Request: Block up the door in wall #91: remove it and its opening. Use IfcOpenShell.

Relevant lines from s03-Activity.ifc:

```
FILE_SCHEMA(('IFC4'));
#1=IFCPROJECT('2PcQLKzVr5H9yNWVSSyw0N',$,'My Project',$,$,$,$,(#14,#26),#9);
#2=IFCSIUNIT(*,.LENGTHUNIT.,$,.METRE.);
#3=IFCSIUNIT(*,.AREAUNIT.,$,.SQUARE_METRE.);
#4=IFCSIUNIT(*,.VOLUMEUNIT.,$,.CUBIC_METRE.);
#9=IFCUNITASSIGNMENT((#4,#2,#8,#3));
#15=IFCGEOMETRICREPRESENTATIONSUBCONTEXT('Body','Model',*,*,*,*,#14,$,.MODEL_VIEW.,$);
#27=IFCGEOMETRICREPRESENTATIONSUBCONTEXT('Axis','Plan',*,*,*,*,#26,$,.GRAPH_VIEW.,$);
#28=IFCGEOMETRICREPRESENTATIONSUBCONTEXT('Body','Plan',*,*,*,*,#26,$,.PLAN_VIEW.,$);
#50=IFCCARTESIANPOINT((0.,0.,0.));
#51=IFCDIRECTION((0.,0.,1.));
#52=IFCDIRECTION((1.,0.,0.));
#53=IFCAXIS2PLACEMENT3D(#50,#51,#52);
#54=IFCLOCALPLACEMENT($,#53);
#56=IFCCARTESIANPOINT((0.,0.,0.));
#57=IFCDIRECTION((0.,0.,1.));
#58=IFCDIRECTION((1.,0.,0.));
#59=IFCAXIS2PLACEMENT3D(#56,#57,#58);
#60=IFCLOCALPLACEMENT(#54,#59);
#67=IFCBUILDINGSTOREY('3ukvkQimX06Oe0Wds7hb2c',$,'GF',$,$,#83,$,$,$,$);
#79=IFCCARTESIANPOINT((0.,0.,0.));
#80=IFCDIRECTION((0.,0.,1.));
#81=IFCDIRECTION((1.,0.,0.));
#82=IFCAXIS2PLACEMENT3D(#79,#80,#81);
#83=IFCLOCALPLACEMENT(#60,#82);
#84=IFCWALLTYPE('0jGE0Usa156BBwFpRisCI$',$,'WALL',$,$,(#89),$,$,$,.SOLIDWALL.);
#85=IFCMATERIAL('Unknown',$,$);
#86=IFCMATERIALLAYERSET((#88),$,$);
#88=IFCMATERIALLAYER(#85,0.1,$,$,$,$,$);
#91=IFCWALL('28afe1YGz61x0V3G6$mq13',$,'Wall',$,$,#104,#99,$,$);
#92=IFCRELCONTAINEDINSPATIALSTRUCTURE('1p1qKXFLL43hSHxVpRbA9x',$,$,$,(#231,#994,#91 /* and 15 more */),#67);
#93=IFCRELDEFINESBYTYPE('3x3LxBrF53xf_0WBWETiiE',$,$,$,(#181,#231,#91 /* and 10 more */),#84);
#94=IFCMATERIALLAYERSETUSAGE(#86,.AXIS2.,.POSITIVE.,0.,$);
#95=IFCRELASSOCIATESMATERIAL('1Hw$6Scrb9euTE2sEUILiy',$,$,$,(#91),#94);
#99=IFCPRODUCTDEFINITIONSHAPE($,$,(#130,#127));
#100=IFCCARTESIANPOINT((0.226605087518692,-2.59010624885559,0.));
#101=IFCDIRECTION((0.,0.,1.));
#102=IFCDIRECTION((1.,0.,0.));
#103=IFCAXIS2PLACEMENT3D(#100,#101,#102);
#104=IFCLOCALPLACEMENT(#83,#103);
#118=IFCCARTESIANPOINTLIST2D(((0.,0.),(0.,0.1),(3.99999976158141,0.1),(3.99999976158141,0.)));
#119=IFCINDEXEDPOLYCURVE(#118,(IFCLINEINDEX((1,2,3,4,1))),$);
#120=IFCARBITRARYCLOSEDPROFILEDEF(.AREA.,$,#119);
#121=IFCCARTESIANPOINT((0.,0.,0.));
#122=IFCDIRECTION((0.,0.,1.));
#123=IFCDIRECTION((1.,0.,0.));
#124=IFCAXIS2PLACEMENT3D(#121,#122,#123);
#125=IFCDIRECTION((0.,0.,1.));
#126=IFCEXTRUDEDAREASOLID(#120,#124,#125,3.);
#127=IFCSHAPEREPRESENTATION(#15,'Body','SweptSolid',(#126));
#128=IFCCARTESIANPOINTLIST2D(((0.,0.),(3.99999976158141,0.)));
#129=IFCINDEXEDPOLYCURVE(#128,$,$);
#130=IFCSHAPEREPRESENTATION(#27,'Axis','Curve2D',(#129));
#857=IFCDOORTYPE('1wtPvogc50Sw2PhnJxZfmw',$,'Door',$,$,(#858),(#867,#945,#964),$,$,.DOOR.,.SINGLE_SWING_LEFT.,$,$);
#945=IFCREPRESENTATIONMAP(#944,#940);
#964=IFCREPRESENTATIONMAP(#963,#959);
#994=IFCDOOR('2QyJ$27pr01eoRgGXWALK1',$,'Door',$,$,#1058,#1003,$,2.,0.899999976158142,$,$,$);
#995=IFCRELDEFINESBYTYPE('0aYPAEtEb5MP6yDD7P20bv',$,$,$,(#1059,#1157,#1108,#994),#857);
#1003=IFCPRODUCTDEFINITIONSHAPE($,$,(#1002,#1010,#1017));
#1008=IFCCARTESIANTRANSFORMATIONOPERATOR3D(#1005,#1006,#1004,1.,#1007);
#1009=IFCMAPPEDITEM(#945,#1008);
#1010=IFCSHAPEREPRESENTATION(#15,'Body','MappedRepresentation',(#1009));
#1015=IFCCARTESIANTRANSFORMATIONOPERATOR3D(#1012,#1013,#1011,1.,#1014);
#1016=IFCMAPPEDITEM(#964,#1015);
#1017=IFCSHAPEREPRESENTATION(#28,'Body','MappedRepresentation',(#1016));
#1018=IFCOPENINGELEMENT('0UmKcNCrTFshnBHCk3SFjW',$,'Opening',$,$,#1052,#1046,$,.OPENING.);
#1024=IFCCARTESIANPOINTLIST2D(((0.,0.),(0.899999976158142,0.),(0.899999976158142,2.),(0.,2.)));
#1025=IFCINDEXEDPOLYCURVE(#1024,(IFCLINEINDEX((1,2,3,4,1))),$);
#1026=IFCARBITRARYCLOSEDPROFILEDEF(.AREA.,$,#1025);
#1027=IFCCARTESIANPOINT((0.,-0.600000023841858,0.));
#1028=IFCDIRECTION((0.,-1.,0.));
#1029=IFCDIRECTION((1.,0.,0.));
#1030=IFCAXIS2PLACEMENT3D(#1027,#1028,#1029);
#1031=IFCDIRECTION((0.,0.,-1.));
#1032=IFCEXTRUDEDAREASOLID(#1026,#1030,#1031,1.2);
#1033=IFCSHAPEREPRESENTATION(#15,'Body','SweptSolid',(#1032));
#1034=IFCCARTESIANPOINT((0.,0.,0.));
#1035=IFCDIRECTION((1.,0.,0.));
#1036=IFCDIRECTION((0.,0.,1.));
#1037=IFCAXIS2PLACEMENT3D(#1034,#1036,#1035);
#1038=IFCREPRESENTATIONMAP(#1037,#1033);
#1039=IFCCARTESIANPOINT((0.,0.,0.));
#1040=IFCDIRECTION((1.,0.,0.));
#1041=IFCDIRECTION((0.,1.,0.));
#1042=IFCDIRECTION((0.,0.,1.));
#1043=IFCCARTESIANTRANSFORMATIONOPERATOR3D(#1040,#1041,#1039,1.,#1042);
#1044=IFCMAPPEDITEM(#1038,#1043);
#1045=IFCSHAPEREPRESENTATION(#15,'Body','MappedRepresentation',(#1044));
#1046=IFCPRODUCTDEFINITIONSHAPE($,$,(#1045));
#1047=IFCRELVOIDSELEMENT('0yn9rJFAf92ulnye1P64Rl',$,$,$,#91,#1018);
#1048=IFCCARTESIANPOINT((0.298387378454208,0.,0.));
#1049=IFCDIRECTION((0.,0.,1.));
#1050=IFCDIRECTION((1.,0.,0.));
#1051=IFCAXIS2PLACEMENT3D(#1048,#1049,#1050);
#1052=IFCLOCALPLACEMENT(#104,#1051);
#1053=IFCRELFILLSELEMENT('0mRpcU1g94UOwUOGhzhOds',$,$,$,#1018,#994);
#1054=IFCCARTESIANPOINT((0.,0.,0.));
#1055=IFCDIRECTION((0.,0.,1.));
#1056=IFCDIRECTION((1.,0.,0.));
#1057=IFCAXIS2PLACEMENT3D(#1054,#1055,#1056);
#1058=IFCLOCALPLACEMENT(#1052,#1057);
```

```python
import ifcopenshell
import ifcopenshell.api.feature
import ifcopenshell.api.root
import ifcopenshell.geom
import ifcopenshell.util.shape

model = ifcopenshell.open("s03-Activity.ifc")
settings = ifcopenshell.geom.settings()


def volume(element):
    """Net volume in cubic metres, openings subtracted."""
    shape = ifcopenshell.geom.create_shape(settings, element)
    return ifcopenshell.util.shape.get_volume(shape.geometry)


door = model.by_guid("2QyJ$27pr01eoRgGXWALK1")
opening = door.FillsVoids[0].RelatingOpeningElement
wall = opening.VoidsElements[0].RelatingBuildingElement
before = volume(wall)

ifcopenshell.api.root.remove_product(model, product=door)
ifcopenshell.api.feature.remove_feature(model, feature=opening)

after = volume(wall)

print(f"wall volume {before:.3f} -> {after:.3f} m3")

model.write("s03-Activity_edited.ifc")
```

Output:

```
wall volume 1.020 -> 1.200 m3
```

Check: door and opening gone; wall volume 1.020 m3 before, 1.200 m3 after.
